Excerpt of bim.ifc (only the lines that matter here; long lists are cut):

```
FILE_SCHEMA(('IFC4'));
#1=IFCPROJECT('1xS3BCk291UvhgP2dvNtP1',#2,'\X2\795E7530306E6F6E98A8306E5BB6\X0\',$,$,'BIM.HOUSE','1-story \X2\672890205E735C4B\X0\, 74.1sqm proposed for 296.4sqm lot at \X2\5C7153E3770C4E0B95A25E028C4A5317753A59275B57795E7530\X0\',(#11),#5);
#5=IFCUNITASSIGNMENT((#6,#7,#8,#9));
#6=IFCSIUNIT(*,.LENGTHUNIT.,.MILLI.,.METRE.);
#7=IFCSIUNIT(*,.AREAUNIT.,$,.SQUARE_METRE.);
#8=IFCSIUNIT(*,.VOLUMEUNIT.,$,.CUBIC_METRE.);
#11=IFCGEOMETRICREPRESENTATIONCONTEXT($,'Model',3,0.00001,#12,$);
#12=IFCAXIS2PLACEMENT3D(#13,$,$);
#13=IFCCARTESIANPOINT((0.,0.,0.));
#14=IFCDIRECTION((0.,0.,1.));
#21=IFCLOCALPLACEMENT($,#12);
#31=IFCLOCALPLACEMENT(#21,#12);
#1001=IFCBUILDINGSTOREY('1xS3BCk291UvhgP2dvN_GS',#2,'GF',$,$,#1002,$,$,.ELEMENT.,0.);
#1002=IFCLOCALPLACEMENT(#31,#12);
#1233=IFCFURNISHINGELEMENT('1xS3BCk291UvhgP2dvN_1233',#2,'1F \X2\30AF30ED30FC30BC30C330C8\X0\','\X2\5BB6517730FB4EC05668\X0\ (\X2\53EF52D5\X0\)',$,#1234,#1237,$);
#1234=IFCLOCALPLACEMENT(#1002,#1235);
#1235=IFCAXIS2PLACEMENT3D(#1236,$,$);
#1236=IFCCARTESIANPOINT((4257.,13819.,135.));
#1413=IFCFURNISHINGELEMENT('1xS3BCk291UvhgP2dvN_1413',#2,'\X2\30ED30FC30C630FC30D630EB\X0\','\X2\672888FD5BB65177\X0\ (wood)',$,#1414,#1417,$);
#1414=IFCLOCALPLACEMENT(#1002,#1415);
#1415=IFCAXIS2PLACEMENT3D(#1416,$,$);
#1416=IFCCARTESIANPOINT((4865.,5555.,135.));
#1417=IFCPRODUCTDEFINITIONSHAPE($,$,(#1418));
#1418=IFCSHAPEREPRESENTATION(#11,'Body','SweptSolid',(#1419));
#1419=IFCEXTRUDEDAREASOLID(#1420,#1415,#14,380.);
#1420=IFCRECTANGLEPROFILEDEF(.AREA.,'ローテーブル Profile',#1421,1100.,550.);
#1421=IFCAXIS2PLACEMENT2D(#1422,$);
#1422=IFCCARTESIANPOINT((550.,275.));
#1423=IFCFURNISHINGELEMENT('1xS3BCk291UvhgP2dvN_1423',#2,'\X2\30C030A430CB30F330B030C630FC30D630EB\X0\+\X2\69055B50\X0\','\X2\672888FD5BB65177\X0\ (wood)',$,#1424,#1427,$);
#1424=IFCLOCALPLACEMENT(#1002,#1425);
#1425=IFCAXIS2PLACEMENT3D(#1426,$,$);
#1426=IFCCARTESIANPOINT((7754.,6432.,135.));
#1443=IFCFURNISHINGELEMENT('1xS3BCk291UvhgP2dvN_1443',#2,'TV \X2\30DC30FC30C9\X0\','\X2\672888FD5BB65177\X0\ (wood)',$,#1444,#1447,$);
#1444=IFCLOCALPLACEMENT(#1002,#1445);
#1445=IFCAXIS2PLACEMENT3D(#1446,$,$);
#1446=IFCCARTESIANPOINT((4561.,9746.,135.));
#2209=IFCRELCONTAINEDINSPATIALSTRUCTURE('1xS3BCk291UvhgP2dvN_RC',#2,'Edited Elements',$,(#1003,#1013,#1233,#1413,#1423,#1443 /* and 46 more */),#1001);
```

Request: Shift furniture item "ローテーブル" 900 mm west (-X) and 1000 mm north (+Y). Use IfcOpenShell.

```python
import ifcopenshell
import ifcopenshell.api.geometry
import ifcopenshell.util.placement
import ifcopenshell.util.unit

model = ifcopenshell.open("bim.ifc")
unit_scale = ifcopenshell.util.unit.calculate_unit_scale(model)

item = model.by_guid("1xS3BCk291UvhgP2dvN_1413")
matrix = ifcopenshell.util.placement.get_local_placement(item.ObjectPlacement)
matrix[0, 3] -= 0.9 / unit_scale
matrix[1, 3] += 1 / unit_scale
ifcopenshell.api.geometry.edit_object_placement(model, product=item, matrix=matrix, is_si=False)

print(ifcopenshell.util.placement.get_local_placement(item.ObjectPlacement).round(3) + 0.0)

model.write("bim_edited.ifc")
```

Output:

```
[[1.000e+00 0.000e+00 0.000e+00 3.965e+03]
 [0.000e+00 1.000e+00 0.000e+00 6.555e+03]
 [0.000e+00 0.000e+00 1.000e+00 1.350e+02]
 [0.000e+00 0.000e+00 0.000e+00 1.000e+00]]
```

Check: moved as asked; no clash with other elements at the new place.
